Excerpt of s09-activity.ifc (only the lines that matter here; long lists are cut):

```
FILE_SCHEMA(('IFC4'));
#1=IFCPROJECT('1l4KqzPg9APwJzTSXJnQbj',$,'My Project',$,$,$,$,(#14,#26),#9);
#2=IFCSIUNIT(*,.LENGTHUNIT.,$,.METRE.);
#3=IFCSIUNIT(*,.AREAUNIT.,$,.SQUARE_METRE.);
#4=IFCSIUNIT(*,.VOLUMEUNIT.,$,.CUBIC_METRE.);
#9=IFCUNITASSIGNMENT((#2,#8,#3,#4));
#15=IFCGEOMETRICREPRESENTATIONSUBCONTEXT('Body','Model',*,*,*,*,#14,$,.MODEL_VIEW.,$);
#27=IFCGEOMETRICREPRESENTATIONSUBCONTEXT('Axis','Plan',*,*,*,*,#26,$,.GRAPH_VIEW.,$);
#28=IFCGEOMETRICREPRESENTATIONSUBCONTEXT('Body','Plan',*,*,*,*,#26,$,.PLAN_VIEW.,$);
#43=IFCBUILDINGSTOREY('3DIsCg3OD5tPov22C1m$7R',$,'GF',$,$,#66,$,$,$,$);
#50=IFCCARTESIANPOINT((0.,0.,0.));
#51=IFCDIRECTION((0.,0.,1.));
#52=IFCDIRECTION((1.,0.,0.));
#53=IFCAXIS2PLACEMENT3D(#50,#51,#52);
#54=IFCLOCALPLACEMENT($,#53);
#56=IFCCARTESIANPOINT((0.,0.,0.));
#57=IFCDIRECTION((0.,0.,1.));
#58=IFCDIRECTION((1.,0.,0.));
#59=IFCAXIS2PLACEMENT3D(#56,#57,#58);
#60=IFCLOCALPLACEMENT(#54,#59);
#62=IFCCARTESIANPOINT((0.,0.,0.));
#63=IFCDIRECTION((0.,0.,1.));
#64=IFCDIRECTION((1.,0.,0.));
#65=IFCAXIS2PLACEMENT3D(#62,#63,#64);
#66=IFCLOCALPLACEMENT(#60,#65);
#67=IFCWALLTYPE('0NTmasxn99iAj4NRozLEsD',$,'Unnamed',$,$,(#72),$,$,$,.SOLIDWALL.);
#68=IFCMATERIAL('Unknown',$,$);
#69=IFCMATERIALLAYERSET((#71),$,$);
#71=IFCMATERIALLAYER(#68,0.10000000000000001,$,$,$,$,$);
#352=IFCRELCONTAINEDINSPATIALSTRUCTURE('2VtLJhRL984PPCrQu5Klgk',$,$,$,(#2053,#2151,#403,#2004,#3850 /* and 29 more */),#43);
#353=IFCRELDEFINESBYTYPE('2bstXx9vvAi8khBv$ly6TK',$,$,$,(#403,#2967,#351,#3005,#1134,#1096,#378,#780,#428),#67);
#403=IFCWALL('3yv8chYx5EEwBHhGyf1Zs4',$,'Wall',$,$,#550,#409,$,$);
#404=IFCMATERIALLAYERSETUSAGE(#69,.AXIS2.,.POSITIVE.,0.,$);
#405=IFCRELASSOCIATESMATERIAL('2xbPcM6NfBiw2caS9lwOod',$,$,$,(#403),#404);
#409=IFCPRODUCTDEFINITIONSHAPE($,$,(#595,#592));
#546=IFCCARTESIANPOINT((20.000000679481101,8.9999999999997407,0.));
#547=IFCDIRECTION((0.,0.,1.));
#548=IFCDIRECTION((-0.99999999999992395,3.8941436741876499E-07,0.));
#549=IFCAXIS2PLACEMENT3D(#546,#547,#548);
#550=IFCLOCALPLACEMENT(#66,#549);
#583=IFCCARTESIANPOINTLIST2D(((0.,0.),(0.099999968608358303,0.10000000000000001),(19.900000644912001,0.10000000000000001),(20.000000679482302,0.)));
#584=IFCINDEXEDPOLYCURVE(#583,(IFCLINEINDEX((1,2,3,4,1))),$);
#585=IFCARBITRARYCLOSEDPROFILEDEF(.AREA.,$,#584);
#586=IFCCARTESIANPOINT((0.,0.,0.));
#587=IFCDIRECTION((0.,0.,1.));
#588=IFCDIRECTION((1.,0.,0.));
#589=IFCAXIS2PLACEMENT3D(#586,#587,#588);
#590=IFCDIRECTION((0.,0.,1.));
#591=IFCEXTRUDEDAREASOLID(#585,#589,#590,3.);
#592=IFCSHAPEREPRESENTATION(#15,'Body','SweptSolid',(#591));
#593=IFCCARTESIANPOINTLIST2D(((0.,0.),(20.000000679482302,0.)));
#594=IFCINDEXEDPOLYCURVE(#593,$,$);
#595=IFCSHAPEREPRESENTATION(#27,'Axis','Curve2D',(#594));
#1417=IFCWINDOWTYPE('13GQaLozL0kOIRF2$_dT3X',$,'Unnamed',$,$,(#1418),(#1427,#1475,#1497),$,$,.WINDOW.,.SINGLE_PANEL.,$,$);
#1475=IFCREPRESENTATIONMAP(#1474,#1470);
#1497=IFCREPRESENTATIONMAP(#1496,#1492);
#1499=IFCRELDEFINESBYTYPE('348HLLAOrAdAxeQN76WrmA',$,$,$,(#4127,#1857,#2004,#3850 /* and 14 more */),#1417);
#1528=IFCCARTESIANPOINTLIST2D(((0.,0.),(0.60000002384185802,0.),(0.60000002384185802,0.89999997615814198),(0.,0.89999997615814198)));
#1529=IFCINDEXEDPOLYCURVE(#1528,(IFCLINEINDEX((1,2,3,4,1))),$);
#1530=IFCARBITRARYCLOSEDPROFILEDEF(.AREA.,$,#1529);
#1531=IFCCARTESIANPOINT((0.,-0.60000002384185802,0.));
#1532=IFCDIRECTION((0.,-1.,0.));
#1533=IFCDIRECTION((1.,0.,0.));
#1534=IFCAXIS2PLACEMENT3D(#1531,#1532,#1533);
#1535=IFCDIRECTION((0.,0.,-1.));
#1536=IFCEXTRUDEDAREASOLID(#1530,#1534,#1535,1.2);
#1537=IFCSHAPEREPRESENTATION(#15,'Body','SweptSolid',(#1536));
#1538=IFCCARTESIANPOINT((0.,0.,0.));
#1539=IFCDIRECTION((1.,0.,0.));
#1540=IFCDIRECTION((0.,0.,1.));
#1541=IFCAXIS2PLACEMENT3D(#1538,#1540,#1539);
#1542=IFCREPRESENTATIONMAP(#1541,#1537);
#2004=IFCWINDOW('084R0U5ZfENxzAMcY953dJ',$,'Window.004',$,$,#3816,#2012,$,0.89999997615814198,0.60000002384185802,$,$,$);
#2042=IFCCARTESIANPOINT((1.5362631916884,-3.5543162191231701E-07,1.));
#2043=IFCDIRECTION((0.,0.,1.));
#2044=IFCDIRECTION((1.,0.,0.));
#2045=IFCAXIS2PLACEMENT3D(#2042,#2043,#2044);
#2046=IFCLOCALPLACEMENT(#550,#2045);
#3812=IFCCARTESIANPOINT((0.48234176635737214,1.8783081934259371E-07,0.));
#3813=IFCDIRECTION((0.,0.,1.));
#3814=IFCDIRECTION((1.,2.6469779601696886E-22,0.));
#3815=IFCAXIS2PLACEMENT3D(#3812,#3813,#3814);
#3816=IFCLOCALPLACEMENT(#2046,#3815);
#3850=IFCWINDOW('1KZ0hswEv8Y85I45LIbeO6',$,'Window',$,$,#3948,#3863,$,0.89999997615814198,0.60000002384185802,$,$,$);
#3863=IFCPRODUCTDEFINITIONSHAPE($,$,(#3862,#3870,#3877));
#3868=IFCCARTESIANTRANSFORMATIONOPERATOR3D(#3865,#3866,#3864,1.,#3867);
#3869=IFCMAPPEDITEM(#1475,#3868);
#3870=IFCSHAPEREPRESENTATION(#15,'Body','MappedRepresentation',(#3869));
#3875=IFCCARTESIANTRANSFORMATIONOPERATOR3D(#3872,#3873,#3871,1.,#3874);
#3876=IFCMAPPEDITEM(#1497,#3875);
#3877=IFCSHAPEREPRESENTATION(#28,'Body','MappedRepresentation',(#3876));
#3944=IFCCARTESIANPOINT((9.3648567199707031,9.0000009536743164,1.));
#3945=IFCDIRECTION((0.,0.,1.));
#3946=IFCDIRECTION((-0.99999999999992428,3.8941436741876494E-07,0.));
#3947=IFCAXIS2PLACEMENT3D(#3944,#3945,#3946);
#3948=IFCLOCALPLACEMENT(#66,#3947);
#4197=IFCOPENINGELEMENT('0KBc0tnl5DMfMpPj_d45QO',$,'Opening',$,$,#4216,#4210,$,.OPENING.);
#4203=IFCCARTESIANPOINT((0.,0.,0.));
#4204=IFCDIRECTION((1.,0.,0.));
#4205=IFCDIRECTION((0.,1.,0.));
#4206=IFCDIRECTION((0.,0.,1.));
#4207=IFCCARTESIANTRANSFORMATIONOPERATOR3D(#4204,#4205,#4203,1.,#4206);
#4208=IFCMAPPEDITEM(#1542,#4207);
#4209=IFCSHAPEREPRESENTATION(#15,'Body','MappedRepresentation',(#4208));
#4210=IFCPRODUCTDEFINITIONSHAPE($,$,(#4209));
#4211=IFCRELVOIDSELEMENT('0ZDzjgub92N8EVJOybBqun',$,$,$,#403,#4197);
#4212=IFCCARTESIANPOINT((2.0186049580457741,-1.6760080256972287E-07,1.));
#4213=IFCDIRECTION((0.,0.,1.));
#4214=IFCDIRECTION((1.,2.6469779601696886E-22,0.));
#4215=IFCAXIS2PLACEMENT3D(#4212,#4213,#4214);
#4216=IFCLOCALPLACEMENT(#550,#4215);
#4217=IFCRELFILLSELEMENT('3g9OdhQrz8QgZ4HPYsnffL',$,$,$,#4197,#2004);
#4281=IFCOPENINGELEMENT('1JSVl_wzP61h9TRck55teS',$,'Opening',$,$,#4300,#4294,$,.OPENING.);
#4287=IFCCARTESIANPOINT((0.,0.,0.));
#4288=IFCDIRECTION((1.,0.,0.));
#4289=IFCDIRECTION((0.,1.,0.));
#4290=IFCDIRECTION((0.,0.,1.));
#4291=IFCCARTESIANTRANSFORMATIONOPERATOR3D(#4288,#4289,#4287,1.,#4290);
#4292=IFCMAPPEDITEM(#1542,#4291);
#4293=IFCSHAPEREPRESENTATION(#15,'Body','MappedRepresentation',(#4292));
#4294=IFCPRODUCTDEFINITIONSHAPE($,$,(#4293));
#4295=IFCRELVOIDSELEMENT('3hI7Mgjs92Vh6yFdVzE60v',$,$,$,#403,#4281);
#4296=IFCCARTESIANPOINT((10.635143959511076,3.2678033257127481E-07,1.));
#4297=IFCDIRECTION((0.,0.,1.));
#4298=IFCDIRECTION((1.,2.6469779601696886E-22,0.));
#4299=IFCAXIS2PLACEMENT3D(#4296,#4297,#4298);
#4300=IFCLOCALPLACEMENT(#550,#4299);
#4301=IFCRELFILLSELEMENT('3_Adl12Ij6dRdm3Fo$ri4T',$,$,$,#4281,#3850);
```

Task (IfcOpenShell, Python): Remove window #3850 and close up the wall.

```python
import ifcopenshell
import ifcopenshell.api.feature
import ifcopenshell.api.root
import ifcopenshell.geom
import ifcopenshell.util.shape

model = ifcopenshell.open("s09-activity.ifc")
settings = ifcopenshell.geom.settings()


def volume(element):
    """Net volume in cubic metres, openings subtracted."""
    shape = ifcopenshell.geom.create_shape(settings, element)
    return ifcopenshell.util.shape.get_volume(shape.geometry)


window = model.by_guid("1KZ0hswEv8Y85I45LIbeO6")
opening = window.FillsVoids[0].RelatingOpeningElement
wall = opening.VoidsElements[0].RelatingBuildingElement
before = volume(wall)

ifcopenshell.api.root.remove_product(model, product=window)
ifcopenshell.api.feature.remove_feature(model, feature=opening)

after = volume(wall)

print(f"wall volume {before:.3f} -> {after:.3f} m3")

model.write("s09-activity-out.ifc")
```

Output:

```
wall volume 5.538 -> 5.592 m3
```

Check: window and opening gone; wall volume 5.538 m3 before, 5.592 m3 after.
